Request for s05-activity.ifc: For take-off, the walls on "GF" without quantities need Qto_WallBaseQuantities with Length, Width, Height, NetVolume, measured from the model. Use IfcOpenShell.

First a look at what the model holds.

```python
import ifcopenshell
import ifcopenshell.util.element
import ifcopenshell.util.unit

model = ifcopenshell.open("s05-activity.ifc")
print(model.schema)
for unit_type in ("LENGTHUNIT", "AREAUNIT", "VOLUMEUNIT"):
    print(unit_type, ifcopenshell.util.unit.calculate_unit_scale(model, unit_type))
storey = next(s for s in model.by_type("IfcBuildingStorey") if s.Name == "GF")
walls = [e for e in ifcopenshell.util.element.get_decomposition(storey) if e.is_a("IfcWall")]
for e in sorted(walls, key=lambda e: e.id()):
    print(e.id(), e.is_a(), e.Name, list(ifcopenshell.util.element.get_psets(e, qtos_only=True)), sep=" | ")
```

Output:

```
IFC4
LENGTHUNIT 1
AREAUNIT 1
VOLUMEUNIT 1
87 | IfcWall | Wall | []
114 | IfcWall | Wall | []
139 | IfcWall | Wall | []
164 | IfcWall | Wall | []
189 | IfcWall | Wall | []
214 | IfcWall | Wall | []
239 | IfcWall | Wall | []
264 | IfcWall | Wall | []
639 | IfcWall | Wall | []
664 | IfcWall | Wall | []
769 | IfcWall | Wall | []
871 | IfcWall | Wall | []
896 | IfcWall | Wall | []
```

```python
import ifcopenshell
import ifcopenshell.api.pset
import ifcopenshell.geom
import ifcopenshell.util.element
import ifcopenshell.util.shape
import ifcopenshell.util.unit

model = ifcopenshell.open("s05-activity.ifc")
unit_scale = ifcopenshell.util.unit.calculate_unit_scale(model)
volume_scale = ifcopenshell.util.unit.calculate_unit_scale(model, "VOLUMEUNIT")
settings = ifcopenshell.geom.settings()

storey = next(s for s in model.by_type("IfcBuildingStorey") if s.Name == "GF")
walls = [e for e in ifcopenshell.util.element.get_decomposition(storey) if e.is_a("IfcWall")]

for e in sorted(walls, key=lambda e: e.id()):
    if ifcopenshell.util.element.get_psets(e, qtos_only=True, should_inherit=False):
        continue
    # Geometry comes back in metres, in the element's own axes.
    shape = ifcopenshell.geom.create_shape(settings, e)
    values = {
        "Length": ifcopenshell.util.shape.get_x(shape.geometry) / unit_scale,
        "Width": ifcopenshell.util.shape.get_y(shape.geometry) / unit_scale,
        "Height": ifcopenshell.util.shape.get_z(shape.geometry) / unit_scale,
        "NetVolume": ifcopenshell.util.shape.get_volume(shape.geometry) / volume_scale,
    }
    qto = ifcopenshell.api.pset.add_qto(model, product=e, name="Qto_WallBaseQuantities")
    ifcopenshell.api.pset.edit_qto(model, qto=qto, properties=values)
    print(e.id(), {k: round(v, 3) for k, v in values.items()})

model.write("s05-activity_edited.ifc")
```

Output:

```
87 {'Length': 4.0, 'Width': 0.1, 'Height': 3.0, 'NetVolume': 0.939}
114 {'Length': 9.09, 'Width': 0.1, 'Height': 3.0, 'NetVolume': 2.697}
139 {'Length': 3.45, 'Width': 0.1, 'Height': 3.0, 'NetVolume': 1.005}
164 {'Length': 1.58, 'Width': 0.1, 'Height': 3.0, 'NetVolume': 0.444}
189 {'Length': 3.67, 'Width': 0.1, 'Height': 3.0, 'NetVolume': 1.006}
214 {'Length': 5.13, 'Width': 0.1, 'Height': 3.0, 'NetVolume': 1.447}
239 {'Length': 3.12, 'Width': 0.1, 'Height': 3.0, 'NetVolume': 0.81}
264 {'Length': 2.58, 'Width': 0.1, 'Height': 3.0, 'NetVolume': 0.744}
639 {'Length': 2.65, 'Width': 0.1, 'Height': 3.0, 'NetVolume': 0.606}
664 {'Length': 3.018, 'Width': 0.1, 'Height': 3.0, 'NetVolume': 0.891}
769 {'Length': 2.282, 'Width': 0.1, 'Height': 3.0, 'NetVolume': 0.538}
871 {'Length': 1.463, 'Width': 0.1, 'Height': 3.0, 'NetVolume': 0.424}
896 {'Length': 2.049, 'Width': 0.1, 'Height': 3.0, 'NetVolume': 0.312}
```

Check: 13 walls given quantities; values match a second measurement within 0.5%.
